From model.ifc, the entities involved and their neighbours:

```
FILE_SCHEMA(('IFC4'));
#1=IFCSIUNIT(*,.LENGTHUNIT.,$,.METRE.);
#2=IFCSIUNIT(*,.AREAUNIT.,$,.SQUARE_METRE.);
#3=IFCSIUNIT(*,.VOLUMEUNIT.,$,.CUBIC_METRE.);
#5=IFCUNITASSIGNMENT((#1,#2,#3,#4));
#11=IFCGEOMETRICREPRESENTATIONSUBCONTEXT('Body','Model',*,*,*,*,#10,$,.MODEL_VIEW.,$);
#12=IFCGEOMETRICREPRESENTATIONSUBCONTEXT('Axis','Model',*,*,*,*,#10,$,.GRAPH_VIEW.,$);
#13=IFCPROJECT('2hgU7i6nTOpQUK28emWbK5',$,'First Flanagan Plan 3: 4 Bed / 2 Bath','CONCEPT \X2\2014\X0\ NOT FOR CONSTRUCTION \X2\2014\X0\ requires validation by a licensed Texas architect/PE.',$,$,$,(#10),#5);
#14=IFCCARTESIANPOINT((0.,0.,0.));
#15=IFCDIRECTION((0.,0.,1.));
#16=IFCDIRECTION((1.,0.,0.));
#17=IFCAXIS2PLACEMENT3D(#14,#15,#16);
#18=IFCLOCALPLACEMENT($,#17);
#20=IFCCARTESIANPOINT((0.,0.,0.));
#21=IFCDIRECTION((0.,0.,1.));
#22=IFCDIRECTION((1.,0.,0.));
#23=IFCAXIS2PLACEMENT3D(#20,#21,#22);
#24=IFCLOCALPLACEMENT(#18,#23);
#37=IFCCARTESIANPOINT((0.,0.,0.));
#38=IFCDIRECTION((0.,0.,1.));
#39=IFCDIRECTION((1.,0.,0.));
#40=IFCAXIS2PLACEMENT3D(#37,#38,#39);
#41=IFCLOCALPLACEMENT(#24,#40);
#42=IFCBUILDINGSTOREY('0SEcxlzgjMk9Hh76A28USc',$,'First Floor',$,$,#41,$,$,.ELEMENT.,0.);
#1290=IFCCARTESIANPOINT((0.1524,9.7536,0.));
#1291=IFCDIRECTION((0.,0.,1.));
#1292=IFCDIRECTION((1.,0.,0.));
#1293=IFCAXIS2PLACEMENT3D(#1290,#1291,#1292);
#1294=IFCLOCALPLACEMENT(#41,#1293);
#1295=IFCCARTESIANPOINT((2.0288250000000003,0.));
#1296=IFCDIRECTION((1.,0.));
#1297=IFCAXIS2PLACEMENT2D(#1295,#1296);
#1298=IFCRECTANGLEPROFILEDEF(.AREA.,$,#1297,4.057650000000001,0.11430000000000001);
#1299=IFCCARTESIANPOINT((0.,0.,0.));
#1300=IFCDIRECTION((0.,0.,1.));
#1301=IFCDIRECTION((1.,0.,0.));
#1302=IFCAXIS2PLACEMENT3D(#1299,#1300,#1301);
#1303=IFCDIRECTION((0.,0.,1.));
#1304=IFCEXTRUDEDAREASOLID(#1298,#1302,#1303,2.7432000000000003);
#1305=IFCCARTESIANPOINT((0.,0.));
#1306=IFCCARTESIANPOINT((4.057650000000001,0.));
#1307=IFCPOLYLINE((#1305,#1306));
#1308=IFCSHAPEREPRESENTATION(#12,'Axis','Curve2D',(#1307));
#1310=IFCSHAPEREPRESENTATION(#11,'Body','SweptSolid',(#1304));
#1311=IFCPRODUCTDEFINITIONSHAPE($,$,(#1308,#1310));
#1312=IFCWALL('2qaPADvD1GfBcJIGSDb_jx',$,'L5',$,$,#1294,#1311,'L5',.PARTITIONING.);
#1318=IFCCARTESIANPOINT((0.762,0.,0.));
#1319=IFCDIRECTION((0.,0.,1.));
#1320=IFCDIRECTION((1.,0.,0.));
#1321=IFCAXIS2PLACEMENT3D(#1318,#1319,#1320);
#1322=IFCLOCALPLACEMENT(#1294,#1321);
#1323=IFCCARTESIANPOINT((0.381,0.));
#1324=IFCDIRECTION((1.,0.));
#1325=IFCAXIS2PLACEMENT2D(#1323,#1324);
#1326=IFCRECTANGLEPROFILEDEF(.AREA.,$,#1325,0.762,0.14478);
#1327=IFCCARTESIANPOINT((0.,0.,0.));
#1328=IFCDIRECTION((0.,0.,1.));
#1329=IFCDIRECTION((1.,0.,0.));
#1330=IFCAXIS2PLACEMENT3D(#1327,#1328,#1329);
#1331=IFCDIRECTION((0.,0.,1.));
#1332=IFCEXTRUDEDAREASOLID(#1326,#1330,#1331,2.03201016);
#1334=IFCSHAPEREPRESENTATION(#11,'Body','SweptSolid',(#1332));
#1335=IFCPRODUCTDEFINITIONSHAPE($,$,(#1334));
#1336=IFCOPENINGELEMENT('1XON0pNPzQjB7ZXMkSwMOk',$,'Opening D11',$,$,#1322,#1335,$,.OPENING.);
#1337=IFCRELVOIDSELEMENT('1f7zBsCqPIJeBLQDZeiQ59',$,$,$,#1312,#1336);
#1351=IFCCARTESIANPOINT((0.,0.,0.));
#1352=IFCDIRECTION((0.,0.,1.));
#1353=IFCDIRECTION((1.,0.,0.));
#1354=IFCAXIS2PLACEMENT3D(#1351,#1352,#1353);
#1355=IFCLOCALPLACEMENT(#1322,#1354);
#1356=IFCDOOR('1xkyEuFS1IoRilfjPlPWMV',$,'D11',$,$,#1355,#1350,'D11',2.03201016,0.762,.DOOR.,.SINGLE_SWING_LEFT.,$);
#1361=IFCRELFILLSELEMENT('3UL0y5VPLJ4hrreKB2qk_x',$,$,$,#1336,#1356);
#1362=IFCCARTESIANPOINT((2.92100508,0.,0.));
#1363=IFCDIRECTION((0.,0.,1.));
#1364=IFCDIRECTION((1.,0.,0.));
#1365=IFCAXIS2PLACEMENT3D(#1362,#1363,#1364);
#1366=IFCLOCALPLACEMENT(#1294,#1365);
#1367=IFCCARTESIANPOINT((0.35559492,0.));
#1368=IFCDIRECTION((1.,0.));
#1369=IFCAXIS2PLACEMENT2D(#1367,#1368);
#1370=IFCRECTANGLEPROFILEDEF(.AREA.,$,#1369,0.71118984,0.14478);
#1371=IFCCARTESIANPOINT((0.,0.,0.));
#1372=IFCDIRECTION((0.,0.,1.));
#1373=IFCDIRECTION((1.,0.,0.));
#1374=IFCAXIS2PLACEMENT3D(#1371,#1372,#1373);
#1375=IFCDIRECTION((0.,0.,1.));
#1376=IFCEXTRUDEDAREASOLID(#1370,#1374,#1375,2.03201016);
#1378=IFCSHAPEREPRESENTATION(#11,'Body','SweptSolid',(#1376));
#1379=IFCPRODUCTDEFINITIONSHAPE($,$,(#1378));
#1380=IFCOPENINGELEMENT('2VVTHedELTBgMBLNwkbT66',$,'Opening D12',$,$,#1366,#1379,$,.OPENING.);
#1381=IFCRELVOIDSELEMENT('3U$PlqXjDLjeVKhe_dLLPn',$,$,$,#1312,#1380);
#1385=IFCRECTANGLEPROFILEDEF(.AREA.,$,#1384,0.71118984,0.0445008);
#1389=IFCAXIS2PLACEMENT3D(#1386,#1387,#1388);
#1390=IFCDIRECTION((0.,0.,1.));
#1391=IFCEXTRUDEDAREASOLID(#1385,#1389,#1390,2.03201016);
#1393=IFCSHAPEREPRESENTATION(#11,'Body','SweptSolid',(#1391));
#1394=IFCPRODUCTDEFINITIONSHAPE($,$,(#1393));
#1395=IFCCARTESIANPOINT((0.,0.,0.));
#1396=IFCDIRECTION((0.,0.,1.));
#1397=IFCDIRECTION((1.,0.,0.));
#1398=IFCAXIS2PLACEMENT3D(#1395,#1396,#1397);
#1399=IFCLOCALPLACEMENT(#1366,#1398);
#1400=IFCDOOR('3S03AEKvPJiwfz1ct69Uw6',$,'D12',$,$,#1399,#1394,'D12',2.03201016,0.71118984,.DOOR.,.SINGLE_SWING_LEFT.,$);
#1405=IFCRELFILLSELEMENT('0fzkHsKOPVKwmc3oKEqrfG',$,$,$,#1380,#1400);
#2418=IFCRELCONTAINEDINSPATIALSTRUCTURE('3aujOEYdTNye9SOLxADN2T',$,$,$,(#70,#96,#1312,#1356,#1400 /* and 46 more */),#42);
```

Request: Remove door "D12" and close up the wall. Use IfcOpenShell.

```python
import ifcopenshell
import ifcopenshell.api.feature
import ifcopenshell.api.root
import ifcopenshell.geom
import ifcopenshell.util.shape

model = ifcopenshell.open("model.ifc")
settings = ifcopenshell.geom.settings()


def volume(element):
    """Net volume in cubic metres, openings subtracted."""
    shape = ifcopenshell.geom.create_shape(settings, element)
    return ifcopenshell.util.shape.get_volume(shape.geometry)


door = model.by_id(1400)
opening = door.FillsVoids[0].RelatingOpeningElement
wall = opening.VoidsElements[0].RelatingBuildingElement
before = volume(wall)

ifcopenshell.api.root.remove_product(model, product=door)
ifcopenshell.api.feature.remove_feature(model, feature=opening)

after = volume(wall)

print(f"wall volume {before:.3f} -> {after:.3f} m3")

model.write("model_v2.ifc")
```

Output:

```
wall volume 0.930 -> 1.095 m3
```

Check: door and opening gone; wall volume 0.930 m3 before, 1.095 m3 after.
